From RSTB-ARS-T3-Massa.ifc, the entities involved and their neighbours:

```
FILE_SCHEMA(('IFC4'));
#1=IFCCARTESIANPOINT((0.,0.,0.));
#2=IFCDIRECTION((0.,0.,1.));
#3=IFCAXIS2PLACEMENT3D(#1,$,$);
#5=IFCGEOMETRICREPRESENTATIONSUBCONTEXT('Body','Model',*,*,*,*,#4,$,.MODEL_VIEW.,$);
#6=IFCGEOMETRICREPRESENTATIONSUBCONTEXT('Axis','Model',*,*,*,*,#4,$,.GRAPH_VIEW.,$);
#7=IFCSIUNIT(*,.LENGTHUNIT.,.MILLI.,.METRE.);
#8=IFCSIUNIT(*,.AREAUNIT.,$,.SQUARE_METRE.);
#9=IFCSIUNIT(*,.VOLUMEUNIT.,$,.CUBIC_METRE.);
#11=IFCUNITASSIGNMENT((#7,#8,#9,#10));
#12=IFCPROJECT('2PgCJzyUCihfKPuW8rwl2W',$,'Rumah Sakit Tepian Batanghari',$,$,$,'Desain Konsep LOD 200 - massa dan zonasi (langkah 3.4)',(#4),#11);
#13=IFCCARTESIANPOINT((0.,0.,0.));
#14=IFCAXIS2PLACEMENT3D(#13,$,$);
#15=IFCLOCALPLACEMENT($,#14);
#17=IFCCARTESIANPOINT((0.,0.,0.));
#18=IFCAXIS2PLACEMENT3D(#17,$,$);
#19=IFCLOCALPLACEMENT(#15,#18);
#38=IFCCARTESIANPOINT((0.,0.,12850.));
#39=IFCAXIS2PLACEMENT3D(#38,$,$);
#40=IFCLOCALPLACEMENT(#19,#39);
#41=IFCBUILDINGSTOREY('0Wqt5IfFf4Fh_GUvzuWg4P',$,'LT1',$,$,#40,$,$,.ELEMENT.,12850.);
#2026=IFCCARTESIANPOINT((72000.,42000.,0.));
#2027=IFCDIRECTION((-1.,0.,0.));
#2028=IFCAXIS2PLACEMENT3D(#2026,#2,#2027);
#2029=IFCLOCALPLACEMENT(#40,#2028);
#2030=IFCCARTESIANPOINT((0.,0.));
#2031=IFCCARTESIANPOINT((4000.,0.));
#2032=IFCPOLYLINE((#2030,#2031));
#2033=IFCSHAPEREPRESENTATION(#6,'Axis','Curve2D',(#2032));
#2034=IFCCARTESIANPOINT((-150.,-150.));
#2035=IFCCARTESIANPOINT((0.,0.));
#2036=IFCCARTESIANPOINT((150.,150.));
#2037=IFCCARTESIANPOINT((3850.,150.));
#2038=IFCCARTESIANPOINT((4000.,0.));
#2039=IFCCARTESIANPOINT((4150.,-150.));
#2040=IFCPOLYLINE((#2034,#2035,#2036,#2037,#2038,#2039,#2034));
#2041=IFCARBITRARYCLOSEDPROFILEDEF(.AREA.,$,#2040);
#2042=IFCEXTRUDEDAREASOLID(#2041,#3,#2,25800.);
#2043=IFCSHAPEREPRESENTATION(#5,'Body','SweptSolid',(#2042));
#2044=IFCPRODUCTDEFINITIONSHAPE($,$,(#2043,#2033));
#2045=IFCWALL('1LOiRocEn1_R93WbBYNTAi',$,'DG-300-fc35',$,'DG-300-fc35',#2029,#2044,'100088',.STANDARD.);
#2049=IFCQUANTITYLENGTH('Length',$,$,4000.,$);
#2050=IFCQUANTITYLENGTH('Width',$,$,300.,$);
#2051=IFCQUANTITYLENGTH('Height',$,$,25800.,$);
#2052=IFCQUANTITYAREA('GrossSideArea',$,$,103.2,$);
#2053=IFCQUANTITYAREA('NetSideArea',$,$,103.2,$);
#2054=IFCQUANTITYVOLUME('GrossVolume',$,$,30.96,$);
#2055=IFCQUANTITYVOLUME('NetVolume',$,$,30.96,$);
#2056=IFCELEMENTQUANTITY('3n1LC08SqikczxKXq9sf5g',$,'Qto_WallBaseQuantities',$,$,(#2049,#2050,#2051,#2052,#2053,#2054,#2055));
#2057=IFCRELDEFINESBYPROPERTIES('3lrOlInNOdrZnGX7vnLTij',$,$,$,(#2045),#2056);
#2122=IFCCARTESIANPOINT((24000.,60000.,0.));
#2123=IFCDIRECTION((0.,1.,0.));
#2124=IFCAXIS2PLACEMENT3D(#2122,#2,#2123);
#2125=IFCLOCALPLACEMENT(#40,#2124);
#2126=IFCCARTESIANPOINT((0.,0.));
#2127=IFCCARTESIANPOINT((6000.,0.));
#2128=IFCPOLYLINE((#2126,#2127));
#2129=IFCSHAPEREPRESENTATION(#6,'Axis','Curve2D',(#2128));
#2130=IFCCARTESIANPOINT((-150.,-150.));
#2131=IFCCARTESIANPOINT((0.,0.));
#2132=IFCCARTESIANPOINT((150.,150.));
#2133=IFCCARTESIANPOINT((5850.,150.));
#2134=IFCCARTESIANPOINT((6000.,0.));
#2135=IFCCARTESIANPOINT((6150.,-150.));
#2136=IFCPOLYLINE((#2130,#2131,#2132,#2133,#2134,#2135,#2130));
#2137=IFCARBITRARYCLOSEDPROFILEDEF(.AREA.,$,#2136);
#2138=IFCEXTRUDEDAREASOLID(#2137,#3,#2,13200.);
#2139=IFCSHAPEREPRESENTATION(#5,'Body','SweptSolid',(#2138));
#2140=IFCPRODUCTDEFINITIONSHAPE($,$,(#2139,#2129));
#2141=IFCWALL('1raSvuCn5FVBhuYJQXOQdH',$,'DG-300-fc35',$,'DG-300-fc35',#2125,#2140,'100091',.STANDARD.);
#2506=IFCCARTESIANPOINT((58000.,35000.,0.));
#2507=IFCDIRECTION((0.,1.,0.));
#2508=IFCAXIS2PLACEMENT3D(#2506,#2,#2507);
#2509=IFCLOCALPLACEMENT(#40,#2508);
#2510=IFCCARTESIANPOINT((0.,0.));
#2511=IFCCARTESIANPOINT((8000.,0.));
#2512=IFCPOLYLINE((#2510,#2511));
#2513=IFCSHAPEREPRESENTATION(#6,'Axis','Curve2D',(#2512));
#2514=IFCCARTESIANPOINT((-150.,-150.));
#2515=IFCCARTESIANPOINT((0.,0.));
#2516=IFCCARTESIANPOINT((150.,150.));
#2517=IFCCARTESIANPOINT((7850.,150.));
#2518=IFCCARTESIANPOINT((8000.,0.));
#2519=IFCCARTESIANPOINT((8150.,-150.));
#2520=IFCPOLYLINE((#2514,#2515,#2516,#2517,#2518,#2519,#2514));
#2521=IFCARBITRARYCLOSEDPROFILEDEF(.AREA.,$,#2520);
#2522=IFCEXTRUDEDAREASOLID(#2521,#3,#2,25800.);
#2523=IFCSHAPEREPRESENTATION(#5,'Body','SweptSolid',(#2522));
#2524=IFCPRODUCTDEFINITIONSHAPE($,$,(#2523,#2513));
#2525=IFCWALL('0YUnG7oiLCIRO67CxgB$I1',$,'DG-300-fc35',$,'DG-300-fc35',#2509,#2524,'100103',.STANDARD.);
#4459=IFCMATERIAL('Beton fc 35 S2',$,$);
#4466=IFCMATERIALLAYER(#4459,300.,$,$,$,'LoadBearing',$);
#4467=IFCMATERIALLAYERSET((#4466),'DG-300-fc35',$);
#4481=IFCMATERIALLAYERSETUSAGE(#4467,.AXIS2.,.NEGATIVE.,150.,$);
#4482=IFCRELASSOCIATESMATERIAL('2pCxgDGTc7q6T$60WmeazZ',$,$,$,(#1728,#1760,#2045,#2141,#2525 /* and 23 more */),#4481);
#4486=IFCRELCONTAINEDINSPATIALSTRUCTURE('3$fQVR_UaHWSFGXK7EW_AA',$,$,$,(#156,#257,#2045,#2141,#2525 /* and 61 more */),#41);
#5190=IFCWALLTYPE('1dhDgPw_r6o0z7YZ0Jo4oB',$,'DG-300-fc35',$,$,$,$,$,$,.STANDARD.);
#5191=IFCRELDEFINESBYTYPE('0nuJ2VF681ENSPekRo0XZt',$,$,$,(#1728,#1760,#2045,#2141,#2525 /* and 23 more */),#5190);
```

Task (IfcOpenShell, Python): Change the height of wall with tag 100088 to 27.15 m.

```python
import ifcopenshell
import ifcopenshell.api.pset
import ifcopenshell.geom
import ifcopenshell.util.element
import ifcopenshell.util.representation
import ifcopenshell.util.shape
import ifcopenshell.util.unit

model = ifcopenshell.open("RSTB-ARS-T3-Massa.ifc")
unit_scale = ifcopenshell.util.unit.calculate_unit_scale(model)
area_scale = ifcopenshell.util.unit.calculate_unit_scale(model, "AREAUNIT")
volume_scale = ifcopenshell.util.unit.calculate_unit_scale(model, "VOLUMEUNIT")
settings = ifcopenshell.geom.settings()


def volume(element):
    """Net volume in cubic metres, openings subtracted."""
    shape = ifcopenshell.geom.create_shape(settings, element)
    return ifcopenshell.util.shape.get_volume(shape.geometry)


wall = model.by_guid("1LOiRocEn1_R93WbBYNTAi")
before = volume(wall)

body = ifcopenshell.util.representation.get_representation(wall, "Model", "Body")
solid = body.Items[0]
old_height = solid.Depth
solid.Depth = 27.15 / unit_scale
after = volume(wall)
thickness = 0.3  # wall thickness in metres

# Update the stored height, areas and volumes.
qto = model.by_id(ifcopenshell.util.element.get_pset(wall, "Qto_WallBaseQuantities", should_inherit=False)["id"])
ifcopenshell.api.pset.edit_qto(model, qto=qto, properties={
    "Height": solid.Depth,
    "GrossSideArea": ifcopenshell.util.element.get_pset(wall, "Qto_WallBaseQuantities", "GrossSideArea") * solid.Depth / old_height,
    "NetSideArea": after / thickness / area_scale,
    "GrossVolume": ifcopenshell.util.element.get_pset(wall, "Qto_WallBaseQuantities", "GrossVolume") * solid.Depth / old_height,
    "NetVolume": after / volume_scale,
})

print(f"height {old_height:g} -> {solid.Depth:g}, volume {before:.3f} -> {after:.3f} m3")

model.write("RSTB-ARS-T3-Massa-out.ifc")
```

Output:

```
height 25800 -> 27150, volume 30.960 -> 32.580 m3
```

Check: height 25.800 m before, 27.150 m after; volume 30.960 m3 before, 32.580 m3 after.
